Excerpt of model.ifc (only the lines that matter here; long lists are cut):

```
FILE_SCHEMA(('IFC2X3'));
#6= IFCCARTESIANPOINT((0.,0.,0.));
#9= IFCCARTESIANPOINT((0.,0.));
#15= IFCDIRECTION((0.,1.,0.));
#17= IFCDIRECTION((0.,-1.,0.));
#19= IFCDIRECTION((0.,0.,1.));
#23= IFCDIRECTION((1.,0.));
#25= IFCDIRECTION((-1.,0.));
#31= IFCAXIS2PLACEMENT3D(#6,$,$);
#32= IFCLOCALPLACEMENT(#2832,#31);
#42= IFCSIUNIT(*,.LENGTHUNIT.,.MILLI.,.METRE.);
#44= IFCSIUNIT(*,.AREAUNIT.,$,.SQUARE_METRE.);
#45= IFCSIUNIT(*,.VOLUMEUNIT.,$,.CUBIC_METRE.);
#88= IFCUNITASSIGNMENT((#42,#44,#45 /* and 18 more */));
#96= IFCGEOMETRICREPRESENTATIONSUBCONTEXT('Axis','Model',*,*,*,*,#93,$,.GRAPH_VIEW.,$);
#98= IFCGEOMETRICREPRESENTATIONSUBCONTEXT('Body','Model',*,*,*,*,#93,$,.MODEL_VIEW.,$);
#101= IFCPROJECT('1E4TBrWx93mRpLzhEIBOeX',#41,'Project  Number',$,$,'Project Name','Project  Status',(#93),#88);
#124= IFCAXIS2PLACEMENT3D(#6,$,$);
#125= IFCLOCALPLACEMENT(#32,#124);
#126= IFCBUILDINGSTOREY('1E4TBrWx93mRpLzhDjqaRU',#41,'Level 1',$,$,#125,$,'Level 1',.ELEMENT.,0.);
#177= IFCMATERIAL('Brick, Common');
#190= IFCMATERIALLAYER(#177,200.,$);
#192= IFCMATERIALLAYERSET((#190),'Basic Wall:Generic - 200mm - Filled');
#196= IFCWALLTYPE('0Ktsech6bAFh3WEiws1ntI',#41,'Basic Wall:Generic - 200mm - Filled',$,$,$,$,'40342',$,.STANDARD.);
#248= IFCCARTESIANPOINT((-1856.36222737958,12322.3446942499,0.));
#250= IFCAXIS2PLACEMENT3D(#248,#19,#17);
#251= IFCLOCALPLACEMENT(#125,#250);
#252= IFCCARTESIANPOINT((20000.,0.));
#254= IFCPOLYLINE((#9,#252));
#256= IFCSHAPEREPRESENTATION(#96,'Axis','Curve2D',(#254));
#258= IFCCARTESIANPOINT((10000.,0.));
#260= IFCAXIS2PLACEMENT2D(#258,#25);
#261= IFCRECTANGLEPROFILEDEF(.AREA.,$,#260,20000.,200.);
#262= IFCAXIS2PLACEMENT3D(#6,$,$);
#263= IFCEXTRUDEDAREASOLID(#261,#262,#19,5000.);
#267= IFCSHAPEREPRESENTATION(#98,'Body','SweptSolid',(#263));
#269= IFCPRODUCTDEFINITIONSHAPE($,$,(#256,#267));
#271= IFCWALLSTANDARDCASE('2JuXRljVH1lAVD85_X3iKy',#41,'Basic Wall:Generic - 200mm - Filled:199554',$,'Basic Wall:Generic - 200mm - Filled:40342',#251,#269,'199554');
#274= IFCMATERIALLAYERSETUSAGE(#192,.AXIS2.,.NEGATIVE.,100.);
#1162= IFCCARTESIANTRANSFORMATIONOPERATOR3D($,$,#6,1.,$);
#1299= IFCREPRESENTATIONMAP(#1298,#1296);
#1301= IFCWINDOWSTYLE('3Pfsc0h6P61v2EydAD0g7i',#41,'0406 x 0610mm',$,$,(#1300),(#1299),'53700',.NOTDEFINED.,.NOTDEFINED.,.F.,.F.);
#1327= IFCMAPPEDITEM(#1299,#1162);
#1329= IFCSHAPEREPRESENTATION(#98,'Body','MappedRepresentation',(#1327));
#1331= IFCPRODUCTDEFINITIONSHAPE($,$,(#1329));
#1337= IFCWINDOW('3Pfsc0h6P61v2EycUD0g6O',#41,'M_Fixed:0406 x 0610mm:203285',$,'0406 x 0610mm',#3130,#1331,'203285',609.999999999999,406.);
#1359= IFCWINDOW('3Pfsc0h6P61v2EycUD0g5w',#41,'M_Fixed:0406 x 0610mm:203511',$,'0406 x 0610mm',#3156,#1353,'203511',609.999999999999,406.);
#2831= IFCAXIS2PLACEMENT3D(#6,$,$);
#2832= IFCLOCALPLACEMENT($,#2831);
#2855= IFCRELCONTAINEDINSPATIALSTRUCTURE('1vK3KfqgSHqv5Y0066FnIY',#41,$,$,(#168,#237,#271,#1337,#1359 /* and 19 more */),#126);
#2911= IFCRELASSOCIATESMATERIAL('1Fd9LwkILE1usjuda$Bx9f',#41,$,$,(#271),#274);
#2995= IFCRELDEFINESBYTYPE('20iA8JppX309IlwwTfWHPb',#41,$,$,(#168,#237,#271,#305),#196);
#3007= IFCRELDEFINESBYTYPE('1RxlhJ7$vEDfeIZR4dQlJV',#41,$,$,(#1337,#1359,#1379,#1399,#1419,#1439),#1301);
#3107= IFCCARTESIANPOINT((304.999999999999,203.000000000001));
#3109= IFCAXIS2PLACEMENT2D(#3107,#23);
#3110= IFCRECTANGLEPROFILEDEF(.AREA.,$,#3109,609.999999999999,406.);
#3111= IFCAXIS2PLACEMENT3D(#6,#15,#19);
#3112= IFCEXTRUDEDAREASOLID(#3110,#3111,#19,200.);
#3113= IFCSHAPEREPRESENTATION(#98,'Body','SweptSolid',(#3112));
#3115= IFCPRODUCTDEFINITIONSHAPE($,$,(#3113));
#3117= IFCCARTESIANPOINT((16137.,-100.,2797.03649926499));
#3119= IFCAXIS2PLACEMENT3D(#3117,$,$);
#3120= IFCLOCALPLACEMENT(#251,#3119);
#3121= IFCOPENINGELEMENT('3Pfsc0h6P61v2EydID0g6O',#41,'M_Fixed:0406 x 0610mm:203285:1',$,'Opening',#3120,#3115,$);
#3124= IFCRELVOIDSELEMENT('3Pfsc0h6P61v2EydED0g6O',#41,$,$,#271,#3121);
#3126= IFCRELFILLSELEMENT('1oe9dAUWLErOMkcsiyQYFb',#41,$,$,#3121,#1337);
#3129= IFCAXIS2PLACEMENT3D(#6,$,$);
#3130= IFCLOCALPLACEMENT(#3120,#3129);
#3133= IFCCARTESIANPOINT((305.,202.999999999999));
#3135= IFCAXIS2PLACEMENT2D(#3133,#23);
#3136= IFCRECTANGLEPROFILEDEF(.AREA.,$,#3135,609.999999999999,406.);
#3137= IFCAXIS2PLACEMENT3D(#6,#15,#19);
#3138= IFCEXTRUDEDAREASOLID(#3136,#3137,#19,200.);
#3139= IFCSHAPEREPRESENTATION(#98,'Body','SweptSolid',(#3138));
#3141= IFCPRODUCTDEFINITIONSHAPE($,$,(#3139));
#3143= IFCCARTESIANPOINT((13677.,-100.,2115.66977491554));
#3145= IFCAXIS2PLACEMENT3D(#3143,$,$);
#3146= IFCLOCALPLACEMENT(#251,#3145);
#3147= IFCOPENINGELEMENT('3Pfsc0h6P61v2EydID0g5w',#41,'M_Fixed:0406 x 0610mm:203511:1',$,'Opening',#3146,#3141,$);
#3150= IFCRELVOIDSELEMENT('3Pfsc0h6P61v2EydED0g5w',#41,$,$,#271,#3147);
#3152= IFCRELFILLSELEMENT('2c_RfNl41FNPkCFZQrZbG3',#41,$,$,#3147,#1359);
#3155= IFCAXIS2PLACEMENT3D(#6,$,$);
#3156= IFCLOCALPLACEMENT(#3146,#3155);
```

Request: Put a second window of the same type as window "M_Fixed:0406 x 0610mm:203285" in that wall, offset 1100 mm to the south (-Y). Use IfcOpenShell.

```python
import ifcopenshell
import ifcopenshell.api.feature
import ifcopenshell.api.geometry
import ifcopenshell.api.root
import ifcopenshell.geom
import ifcopenshell.util.element
import ifcopenshell.util.placement
import ifcopenshell.util.shape

model = ifcopenshell.open("model.ifc")
settings = ifcopenshell.geom.settings()


def volume(element):
    """Net volume in cubic metres, openings subtracted."""
    shape = ifcopenshell.geom.create_shape(settings, element)
    return ifcopenshell.util.shape.get_volume(shape.geometry)


def reuse_history(source, copy):
    """copy_class also copies each property set's owner history, people and application; keep the originals."""
    for rel in copy.IsDefinedBy:
        if rel.is_a("IfcRelDefinesByProperties") and (history := rel.RelatingPropertyDefinition.OwnerHistory):
            rel.RelatingPropertyDefinition.OwnerHistory = source.OwnerHistory
            ifcopenshell.util.element.remove_deep2(model, history)


window = model.by_guid("3Pfsc0h6P61v2EycUD0g6O")
opening = window.FillsVoids[0].RelatingOpeningElement
wall = opening.VoidsElements[0].RelatingBuildingElement
before = volume(wall)
shift = ifcopenshell.util.placement.get_local_placement(wall.ObjectPlacement)[:3, 0] * 1100.0

# copy_class copies the void relationship, type, container and properties, but no geometry.
new_opening = ifcopenshell.api.root.copy_class(model, product=opening)
new_opening.Representation = ifcopenshell.util.element.copy_deep(
    model, opening.Representation, exclude=["IfcGeometricRepresentationContext", "IfcRepresentationMap"]
)
new_opening.Name = "M_Fixed:0406 x 0610mm"
new_window = ifcopenshell.api.root.copy_class(model, product=window)
new_window.Representation = ifcopenshell.util.element.copy_deep(
    model, window.Representation, exclude=["IfcGeometricRepresentationContext", "IfcRepresentationMap"]
)
new_window.Name = "M_Fixed:0406 x 0610mm"
new_window.Tag = None
reuse_history(window, new_window)
fills = ifcopenshell.api.feature.add_filling(model, opening=new_opening, element=new_window)
fills.OwnerHistory = new_window.OwnerHistory  # required in IFC2X3

for old, new in ((opening, new_opening), (window, new_window)):
    matrix = ifcopenshell.util.placement.get_local_placement(old.ObjectPlacement)
    matrix[:3, 3] += shift
    ifcopenshell.api.geometry.edit_object_placement(model, product=new, matrix=matrix, is_si=False)

after = volume(wall)

print(f"wall volume {before:.3f} -> {after:.3f} m3")

model.write("model_v2.ifc")
```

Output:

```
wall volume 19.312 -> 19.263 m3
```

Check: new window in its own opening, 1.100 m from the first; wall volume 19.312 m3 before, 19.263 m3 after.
